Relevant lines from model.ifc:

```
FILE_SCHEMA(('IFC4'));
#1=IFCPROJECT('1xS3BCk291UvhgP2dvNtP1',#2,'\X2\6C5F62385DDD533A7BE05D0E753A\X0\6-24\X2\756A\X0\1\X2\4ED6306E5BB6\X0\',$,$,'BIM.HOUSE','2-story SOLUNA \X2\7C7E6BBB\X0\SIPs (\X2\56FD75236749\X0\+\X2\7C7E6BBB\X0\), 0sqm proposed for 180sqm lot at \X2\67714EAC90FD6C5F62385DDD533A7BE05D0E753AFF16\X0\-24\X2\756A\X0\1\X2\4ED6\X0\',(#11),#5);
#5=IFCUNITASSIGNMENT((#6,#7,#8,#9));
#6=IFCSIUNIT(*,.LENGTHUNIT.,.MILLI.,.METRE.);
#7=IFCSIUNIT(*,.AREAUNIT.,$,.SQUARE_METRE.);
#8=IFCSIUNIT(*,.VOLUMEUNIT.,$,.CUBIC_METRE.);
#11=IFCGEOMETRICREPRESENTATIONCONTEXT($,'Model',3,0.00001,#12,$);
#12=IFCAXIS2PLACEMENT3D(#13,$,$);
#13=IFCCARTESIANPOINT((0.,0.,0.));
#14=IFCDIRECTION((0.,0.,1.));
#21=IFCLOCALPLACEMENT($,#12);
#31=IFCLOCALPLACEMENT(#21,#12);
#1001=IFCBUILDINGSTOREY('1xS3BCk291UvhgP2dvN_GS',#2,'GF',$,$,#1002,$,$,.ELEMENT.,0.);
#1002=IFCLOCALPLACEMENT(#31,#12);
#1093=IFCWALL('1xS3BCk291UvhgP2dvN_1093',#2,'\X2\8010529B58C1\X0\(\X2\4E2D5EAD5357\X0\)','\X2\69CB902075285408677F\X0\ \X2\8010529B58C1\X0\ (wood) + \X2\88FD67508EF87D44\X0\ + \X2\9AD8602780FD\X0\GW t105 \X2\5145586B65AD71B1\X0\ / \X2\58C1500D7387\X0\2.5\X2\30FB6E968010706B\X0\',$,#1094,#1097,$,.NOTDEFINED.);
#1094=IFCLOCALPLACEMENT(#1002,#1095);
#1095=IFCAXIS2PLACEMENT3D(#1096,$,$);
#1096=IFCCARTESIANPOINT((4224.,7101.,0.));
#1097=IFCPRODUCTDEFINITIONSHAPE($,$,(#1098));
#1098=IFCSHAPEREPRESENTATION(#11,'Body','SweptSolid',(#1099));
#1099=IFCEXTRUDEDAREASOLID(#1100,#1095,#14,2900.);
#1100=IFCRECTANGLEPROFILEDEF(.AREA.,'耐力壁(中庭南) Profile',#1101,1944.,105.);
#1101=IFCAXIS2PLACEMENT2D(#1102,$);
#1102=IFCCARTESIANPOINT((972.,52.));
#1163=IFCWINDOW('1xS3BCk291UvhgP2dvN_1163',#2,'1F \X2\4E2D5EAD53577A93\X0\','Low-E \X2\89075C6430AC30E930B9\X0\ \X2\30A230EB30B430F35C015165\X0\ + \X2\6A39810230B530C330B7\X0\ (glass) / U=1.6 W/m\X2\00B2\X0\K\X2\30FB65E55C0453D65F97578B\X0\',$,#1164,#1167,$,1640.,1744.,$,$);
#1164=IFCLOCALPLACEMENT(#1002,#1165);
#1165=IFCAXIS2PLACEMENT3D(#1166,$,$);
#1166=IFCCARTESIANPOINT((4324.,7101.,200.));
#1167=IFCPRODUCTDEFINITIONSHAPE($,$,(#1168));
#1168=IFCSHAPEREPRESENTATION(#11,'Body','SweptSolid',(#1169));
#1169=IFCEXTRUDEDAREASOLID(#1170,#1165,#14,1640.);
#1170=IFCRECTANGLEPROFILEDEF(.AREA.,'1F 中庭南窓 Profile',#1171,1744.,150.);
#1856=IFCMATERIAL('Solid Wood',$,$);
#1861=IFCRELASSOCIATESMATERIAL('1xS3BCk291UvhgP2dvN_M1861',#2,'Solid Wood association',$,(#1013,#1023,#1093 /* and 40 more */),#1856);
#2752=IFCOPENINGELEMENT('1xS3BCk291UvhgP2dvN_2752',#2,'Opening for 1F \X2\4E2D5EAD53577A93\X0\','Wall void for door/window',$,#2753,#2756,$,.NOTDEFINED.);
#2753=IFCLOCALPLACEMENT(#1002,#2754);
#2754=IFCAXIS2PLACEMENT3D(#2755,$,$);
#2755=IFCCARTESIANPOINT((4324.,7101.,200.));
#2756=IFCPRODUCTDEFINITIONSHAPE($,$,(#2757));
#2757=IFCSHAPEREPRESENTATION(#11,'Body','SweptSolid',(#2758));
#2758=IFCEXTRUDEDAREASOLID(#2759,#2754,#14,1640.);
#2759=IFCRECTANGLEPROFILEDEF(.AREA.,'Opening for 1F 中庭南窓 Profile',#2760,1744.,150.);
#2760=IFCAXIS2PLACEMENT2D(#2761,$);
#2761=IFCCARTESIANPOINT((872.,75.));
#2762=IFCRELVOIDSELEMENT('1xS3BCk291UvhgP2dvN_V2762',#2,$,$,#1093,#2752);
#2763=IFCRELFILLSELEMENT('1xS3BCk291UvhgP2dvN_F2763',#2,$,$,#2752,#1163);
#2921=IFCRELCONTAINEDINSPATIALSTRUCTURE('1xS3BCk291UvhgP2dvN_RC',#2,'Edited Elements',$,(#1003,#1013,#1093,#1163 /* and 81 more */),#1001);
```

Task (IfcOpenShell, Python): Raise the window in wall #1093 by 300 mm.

```python
import numpy as np
import ifcopenshell
import ifcopenshell.api.geometry
import ifcopenshell.util.placement
import ifcopenshell.util.unit

model = ifcopenshell.open("model.ifc")
unit_scale = ifcopenshell.util.unit.calculate_unit_scale(model)

window = model.by_id(1163)
opening = window.FillsVoids[0].RelatingOpeningElement
dz = 0.3 / unit_scale

shift = np.array([0.0, 0.0, dz])
# The window is not placed relative to its opening, so move both.
for product in (opening, window):
    matrix = ifcopenshell.util.placement.get_local_placement(product.ObjectPlacement)
    matrix[:3, 3] += shift
    ifcopenshell.api.geometry.edit_object_placement(model, product=product, matrix=matrix, is_si=False)

print(f"moved by {dz * unit_scale:+.3f} m")

model.write("model_v2.ifc")
```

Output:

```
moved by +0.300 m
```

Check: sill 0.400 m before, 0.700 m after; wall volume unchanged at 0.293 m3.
